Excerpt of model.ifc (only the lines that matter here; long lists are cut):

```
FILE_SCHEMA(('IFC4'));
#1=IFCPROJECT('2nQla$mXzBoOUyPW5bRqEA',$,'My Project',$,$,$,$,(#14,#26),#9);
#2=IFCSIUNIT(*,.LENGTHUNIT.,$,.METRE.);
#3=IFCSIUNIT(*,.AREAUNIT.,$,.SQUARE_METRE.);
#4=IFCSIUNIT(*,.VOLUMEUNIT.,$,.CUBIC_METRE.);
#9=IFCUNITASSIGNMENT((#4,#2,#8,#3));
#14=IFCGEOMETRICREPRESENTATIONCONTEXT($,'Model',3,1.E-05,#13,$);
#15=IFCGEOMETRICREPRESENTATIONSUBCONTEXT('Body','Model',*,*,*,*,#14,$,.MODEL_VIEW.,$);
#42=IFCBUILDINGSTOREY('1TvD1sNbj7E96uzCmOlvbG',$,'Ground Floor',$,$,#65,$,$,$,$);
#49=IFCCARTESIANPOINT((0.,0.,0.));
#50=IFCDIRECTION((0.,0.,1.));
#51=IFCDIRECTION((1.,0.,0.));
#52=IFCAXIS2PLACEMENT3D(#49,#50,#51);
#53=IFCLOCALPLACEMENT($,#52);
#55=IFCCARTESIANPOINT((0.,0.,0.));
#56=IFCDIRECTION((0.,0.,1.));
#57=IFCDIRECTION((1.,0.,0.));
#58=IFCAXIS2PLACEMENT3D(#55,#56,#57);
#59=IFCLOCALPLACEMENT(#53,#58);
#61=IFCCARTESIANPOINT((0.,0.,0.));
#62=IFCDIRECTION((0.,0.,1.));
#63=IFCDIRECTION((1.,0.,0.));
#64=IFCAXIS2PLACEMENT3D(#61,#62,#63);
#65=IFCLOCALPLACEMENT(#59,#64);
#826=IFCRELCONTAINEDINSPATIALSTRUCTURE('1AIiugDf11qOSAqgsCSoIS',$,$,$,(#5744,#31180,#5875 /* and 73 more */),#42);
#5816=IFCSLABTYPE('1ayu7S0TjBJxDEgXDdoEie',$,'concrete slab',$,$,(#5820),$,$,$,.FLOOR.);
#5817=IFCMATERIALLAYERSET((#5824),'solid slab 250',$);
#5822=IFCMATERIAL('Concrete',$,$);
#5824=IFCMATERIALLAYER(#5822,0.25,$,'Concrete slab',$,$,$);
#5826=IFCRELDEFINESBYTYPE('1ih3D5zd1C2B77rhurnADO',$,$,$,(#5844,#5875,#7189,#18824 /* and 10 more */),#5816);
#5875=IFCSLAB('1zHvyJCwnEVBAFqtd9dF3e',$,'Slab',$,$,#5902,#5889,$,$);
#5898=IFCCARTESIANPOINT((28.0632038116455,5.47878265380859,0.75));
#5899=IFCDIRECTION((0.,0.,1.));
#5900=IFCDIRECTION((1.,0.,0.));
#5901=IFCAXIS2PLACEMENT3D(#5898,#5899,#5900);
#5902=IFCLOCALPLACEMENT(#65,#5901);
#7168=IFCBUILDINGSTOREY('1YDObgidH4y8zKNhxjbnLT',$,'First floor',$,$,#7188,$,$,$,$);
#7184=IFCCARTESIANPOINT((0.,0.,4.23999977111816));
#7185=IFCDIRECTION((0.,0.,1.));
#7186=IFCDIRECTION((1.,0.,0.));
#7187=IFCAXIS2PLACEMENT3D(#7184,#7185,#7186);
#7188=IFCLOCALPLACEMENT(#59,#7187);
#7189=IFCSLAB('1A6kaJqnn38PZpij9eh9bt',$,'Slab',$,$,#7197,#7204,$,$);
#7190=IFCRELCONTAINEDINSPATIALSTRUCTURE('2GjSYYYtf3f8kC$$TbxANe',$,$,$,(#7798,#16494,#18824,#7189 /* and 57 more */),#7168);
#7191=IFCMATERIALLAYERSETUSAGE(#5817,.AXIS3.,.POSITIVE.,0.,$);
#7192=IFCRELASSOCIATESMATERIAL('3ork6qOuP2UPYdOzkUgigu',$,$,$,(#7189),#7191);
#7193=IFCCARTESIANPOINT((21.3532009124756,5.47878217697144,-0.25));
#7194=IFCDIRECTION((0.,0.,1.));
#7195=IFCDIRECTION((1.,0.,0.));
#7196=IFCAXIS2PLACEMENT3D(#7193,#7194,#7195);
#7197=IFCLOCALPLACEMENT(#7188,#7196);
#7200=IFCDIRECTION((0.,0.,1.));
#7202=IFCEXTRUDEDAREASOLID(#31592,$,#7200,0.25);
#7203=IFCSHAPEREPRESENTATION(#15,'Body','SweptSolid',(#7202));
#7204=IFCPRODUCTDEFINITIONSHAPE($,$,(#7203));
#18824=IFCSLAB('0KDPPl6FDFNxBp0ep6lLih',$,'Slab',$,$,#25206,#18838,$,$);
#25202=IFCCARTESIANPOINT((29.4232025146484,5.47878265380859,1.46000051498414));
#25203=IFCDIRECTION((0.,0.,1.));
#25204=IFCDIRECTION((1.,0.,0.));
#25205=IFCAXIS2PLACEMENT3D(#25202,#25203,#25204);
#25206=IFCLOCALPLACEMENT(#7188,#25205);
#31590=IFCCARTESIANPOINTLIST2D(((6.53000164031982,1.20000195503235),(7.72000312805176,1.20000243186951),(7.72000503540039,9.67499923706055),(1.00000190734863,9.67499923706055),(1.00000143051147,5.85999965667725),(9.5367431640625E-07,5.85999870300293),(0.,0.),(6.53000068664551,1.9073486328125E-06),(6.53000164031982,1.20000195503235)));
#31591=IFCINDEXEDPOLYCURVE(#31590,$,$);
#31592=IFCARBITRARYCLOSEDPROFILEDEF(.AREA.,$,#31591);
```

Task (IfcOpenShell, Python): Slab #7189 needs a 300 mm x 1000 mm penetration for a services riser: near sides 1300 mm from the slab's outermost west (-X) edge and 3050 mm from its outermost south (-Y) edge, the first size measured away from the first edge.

```python
import numpy as np
import ifcopenshell
import ifcopenshell.api.feature
import ifcopenshell.api.geometry
import ifcopenshell.api.root
import ifcopenshell.geom
import ifcopenshell.util.placement
import ifcopenshell.util.representation
import ifcopenshell.util.shape
import ifcopenshell.util.unit

model = ifcopenshell.open("model.ifc")
unit_scale = ifcopenshell.util.unit.calculate_unit_scale(model)
settings = ifcopenshell.geom.settings()


def volume(element):
    """Net volume in cubic metres, openings subtracted."""
    shape = ifcopenshell.geom.create_shape(settings, element)
    return ifcopenshell.util.shape.get_volume(shape.geometry)


slab = model.by_guid("1A6kaJqnn38PZpij9eh9bt")
before = volume(slab)

# Extent in the slab's own axes, in metres. The edges named are its -X and -Y sides.
slab_shape = ifcopenshell.geom.create_shape(settings, slab)
vertices = ifcopenshell.util.shape.get_vertices(slab_shape.geometry)
x_min, y_min, bottom = vertices.min(axis=0)
top = vertices[:, 2].max()

opening = ifcopenshell.api.root.create_entity(model, ifc_class="IfcOpeningElement", name="Services riser opening", predefined_type="OPENING")
context = ifcopenshell.util.representation.get_context(model, "Model", "Body", "MODEL_VIEW")
width, depth = 0.3, 1
outline = [(0.0, 0.0), (width, 0.0), (width, depth), (0.0, depth), (0.0, 0.0)]
# Overshoot both faces by 50 mm so the cut is clean.
shape = ifcopenshell.api.geometry.add_slab_representation(
    model, context=context, depth=top - bottom + 0.1, polyline=outline
)
ifcopenshell.api.geometry.assign_representation(model, product=opening, representation=shape)

matrix = ifcopenshell.util.placement.get_local_placement(slab.ObjectPlacement)
matrix[:, 3] = matrix @ np.append(np.array([x_min + 1.3, y_min + 3.05, bottom - 0.05]) / unit_scale, 1.0)
ifcopenshell.api.geometry.edit_object_placement(model, product=opening, matrix=matrix, is_si=False)
ifcopenshell.api.feature.add_feature(model, feature=opening, element=slab)

after = volume(slab)

print(f"slab volume {before:.3f} -> {after:.3f} m3")

model.write("model_updated.ifc")
```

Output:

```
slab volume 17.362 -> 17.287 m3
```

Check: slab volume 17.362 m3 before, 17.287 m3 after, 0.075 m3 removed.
